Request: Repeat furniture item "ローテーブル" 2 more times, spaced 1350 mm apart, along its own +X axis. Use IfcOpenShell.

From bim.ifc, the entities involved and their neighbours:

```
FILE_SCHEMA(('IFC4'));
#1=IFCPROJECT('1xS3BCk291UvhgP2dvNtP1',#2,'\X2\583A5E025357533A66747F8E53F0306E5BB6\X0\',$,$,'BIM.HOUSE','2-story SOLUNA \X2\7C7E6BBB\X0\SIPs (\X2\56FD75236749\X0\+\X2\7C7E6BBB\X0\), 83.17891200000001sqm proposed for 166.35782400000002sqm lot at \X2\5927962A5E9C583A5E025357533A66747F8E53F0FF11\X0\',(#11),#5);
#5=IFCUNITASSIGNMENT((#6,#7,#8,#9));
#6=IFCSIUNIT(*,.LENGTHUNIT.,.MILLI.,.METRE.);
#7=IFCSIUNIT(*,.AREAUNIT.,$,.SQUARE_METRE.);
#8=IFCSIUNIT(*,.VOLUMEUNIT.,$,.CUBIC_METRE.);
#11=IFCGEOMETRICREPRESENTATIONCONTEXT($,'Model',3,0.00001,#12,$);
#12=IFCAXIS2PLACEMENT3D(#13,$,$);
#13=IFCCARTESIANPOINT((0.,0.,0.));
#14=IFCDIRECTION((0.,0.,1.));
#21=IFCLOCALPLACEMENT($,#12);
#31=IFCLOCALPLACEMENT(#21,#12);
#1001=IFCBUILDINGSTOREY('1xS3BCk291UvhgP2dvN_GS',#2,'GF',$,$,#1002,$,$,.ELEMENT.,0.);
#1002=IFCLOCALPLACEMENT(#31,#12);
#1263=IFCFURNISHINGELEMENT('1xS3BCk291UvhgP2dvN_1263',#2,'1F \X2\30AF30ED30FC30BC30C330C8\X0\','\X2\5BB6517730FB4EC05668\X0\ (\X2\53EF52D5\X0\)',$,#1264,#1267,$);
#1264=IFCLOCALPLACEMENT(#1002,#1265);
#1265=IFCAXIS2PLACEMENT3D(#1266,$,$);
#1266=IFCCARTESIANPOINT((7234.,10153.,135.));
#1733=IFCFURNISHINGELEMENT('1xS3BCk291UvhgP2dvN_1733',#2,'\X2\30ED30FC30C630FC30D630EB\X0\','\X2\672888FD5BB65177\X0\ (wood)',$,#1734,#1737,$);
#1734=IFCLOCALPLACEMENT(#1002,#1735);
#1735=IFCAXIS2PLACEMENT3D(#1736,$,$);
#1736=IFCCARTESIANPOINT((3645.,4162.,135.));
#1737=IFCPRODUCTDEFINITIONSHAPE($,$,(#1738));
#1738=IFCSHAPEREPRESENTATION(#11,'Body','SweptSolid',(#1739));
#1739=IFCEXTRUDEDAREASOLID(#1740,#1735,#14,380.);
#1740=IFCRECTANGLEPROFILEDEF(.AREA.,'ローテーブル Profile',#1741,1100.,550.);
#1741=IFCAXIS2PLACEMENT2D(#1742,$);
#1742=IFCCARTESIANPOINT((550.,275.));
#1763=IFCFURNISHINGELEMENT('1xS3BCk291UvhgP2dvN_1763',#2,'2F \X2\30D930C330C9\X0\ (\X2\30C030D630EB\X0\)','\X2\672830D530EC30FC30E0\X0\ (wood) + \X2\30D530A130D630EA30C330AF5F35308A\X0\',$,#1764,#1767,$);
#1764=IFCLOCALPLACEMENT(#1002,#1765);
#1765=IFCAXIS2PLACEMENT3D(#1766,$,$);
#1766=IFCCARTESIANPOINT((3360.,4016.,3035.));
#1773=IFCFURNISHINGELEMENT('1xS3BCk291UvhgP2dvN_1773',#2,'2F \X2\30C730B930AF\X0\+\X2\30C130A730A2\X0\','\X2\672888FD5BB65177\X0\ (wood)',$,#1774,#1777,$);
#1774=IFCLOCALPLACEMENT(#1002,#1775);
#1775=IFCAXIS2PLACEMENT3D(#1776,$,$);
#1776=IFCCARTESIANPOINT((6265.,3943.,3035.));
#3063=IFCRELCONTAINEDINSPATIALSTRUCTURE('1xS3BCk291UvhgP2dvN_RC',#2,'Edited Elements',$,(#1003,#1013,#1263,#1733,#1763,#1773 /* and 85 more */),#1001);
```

```python
import ifcopenshell
import ifcopenshell.api.geometry
import ifcopenshell.api.root
import ifcopenshell.util.element
import ifcopenshell.util.placement
import ifcopenshell.util.unit

model = ifcopenshell.open("bim.ifc")
unit_scale = ifcopenshell.util.unit.calculate_unit_scale(model)


def reuse_history(source, copy):
    """copy_class also copies each property set's owner history, people and application; keep the originals."""
    for rel in copy.IsDefinedBy:
        if rel.is_a("IfcRelDefinesByProperties") and (history := rel.RelatingPropertyDefinition.OwnerHistory):
            rel.RelatingPropertyDefinition.OwnerHistory = source.OwnerHistory
            ifcopenshell.util.element.remove_deep2(model, history)


source = model.by_guid("1xS3BCk291UvhgP2dvN_1733")
base = ifcopenshell.util.placement.get_local_placement(source.ObjectPlacement)
step = base[:3, 0] * 1.35 / unit_scale

for i in range(1, 3):
    copy = ifcopenshell.api.root.copy_class(model, product=source)
    copy.Representation = ifcopenshell.util.element.copy_deep(
        model, source.Representation, exclude=["IfcGeometricRepresentationContext", "IfcRepresentationMap"]
    )
    reuse_history(source, copy)
    matrix = base.copy()
    matrix[:3, 3] += i * step
    print("added at", matrix[:3, 3].round(3) + 0.0)
    ifcopenshell.api.geometry.edit_object_placement(model, product=copy, matrix=matrix, is_si=False)

model.write("bim_rev.ifc")
```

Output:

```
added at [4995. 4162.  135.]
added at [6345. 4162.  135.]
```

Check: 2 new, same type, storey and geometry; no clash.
